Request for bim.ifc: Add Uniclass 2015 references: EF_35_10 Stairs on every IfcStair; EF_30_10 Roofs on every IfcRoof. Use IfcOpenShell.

First a look at what the model holds.

```python
import ifcopenshell

model = ifcopenshell.open("bim.ifc")
print(model.schema)
print("classifications:", [c.Name for c in model.by_type("IfcClassification")])
for ifc_class in ("IfcDoor", "IfcRoof", "IfcStair", "IfcWall", "IfcWindow"):
    print(ifc_class, len(model.by_type(ifc_class)))
```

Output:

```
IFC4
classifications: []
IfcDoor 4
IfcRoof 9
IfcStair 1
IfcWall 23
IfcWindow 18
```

```python
import ifcopenshell
import ifcopenshell.api.classification

model = ifcopenshell.open("bim.ifc")

system = ifcopenshell.api.classification.add_classification(model, classification="Uniclass 2015")

codes = {
    "IfcStair": ("EF_35_10", "Stairs"),
    "IfcRoof": ("EF_30_10", "Roofs"),
}
for ifc_class, (code, name) in codes.items():
    products = model.by_type(ifc_class)
    ifcopenshell.api.classification.add_reference(
        model, products=products, classification=system, identification=code, name=name
    )
    print(code, len(products))

model.write("bim_edited.ifc")
```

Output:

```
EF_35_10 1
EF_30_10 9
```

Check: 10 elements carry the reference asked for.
